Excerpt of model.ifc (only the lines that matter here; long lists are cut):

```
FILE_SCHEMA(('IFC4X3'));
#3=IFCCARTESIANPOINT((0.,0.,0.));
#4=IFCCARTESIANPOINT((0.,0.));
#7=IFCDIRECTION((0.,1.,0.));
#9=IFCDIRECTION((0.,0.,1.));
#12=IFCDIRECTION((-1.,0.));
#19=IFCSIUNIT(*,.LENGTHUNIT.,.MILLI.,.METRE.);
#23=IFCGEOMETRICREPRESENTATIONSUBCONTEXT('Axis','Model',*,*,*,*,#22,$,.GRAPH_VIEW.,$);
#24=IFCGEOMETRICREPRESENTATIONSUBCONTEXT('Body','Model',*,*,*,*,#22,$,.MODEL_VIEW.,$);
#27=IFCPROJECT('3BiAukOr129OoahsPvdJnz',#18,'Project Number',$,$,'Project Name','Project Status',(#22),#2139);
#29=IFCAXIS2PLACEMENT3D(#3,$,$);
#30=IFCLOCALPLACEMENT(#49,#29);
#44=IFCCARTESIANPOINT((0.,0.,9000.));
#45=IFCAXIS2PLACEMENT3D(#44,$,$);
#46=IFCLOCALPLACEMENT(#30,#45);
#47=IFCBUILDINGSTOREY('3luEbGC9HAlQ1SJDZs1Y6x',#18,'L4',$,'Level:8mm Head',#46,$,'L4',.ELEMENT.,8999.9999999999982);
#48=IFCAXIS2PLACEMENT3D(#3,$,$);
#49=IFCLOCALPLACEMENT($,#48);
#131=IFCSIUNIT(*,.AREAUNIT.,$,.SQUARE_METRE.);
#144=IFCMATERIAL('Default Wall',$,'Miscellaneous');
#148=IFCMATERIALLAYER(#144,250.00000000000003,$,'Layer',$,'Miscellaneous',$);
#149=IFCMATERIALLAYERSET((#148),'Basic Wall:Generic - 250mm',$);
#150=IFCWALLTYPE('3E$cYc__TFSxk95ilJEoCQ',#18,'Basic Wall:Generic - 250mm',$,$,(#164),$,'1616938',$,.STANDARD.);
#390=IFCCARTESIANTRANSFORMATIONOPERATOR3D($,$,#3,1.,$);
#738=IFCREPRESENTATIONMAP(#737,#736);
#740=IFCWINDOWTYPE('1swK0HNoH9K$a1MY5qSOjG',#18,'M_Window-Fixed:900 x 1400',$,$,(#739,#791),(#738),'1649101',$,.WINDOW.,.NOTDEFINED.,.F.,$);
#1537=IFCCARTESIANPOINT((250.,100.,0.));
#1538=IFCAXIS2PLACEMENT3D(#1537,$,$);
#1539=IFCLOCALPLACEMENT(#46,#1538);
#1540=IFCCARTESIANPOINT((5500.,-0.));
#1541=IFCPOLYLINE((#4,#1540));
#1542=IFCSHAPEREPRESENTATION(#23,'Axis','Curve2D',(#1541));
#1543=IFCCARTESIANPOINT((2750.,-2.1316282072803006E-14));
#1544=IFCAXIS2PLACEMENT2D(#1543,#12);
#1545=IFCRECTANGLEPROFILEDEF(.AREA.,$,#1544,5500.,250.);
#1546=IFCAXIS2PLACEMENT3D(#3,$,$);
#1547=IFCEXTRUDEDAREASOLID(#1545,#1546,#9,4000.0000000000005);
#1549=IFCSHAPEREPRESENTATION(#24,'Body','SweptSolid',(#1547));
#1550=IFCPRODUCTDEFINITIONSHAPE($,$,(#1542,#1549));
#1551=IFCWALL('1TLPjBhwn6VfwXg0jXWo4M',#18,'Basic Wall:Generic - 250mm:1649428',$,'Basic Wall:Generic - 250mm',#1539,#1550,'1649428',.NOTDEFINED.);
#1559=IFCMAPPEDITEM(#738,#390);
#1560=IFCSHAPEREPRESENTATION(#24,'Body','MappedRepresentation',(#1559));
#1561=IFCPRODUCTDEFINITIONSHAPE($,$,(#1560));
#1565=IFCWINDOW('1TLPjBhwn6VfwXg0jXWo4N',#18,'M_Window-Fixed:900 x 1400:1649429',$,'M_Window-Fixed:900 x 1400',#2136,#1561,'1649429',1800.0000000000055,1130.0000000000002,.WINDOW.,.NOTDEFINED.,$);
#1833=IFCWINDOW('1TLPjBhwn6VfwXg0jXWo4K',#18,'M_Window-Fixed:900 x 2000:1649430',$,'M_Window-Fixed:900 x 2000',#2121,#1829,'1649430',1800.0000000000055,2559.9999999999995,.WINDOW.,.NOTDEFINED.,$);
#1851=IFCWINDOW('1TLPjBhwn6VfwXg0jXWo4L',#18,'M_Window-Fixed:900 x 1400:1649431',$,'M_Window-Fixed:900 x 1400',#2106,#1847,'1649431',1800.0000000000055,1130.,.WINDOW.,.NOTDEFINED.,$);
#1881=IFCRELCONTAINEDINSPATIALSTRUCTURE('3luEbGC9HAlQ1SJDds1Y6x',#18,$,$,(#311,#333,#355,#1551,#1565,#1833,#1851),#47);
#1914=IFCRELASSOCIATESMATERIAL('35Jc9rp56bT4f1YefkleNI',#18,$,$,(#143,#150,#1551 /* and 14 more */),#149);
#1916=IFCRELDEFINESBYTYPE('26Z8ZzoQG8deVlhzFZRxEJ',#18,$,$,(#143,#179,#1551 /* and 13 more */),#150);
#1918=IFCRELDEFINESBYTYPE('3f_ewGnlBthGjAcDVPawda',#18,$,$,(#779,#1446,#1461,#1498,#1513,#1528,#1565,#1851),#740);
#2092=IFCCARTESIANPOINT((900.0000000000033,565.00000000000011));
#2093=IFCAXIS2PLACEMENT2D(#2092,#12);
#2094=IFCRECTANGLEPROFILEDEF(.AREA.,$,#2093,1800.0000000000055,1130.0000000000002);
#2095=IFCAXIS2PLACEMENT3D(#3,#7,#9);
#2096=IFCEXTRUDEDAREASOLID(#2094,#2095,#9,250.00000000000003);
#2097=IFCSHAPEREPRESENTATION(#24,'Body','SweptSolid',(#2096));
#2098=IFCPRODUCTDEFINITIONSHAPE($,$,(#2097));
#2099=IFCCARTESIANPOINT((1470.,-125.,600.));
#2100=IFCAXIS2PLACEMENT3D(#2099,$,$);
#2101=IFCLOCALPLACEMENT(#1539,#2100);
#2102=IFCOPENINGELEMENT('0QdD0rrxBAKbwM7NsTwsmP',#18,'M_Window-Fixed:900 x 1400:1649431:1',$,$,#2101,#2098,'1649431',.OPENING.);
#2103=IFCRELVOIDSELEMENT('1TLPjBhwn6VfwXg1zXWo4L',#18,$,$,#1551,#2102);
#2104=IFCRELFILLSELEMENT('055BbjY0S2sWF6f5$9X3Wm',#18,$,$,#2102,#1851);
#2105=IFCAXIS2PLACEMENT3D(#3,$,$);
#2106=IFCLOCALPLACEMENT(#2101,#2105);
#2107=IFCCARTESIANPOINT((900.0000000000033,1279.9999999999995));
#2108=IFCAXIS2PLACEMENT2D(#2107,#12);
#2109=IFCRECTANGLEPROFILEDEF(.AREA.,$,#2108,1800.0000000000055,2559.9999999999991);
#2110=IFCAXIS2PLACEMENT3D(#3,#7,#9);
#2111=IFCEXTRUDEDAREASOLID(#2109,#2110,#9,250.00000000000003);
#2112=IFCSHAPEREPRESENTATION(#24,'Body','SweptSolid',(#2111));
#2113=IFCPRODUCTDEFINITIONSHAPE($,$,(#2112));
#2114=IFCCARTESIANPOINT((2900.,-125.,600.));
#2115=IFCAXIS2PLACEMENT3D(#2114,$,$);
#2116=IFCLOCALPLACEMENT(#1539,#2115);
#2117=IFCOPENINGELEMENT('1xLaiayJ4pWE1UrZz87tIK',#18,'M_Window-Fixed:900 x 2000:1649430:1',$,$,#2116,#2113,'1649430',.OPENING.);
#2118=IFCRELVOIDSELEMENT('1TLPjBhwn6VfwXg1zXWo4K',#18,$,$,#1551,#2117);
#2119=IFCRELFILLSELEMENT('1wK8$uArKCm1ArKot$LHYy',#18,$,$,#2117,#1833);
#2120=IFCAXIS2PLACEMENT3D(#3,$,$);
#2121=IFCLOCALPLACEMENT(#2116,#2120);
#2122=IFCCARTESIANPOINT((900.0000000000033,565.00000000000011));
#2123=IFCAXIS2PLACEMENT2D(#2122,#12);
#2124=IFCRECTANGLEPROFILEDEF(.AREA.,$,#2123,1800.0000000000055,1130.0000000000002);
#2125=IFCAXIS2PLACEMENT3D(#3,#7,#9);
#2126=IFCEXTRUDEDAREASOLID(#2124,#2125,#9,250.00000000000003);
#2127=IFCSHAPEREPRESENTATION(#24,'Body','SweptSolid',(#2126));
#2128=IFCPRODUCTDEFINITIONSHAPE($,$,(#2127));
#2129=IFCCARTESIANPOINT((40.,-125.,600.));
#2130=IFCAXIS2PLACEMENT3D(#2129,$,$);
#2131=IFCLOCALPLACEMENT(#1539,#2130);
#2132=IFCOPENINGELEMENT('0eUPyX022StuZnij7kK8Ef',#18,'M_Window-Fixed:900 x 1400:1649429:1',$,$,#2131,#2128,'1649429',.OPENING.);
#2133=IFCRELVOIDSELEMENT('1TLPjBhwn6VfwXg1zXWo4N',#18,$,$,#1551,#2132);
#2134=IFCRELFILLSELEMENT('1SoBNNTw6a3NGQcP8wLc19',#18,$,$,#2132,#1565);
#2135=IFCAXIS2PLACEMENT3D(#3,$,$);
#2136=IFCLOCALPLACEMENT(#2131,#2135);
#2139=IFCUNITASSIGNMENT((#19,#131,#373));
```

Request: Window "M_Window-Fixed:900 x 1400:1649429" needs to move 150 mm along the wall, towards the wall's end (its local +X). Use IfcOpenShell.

```python
import ifcopenshell
import ifcopenshell.api.geometry
import ifcopenshell.util.placement
import ifcopenshell.util.unit

model = ifcopenshell.open("model.ifc")
unit_scale = ifcopenshell.util.unit.calculate_unit_scale(model)

window = model.by_id(1565)
opening = window.FillsVoids[0].RelatingOpeningElement
wall = opening.VoidsElements[0].RelatingBuildingElement

wall_matrix = ifcopenshell.util.placement.get_local_placement(wall.ObjectPlacement)
shift = wall_matrix[:3, 0] * 0.15 / unit_scale
before = ifcopenshell.util.placement.get_local_placement(window.ObjectPlacement)[:3, 3].copy()

# The window is placed relative to its opening, so it follows when the opening moves.
matrix = ifcopenshell.util.placement.get_local_placement(opening.ObjectPlacement)
matrix[:3, 3] += shift
ifcopenshell.api.geometry.edit_object_placement(
    model, product=opening, matrix=matrix, is_si=False, should_transform_children=True
)

after = ifcopenshell.util.placement.get_local_placement(window.ObjectPlacement)[:3, 3]
print("window moved by", (after - before).round(3) + 0.0)

model.write("model_updated.ifc")
```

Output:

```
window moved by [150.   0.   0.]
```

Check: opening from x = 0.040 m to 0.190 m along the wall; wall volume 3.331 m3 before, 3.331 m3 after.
